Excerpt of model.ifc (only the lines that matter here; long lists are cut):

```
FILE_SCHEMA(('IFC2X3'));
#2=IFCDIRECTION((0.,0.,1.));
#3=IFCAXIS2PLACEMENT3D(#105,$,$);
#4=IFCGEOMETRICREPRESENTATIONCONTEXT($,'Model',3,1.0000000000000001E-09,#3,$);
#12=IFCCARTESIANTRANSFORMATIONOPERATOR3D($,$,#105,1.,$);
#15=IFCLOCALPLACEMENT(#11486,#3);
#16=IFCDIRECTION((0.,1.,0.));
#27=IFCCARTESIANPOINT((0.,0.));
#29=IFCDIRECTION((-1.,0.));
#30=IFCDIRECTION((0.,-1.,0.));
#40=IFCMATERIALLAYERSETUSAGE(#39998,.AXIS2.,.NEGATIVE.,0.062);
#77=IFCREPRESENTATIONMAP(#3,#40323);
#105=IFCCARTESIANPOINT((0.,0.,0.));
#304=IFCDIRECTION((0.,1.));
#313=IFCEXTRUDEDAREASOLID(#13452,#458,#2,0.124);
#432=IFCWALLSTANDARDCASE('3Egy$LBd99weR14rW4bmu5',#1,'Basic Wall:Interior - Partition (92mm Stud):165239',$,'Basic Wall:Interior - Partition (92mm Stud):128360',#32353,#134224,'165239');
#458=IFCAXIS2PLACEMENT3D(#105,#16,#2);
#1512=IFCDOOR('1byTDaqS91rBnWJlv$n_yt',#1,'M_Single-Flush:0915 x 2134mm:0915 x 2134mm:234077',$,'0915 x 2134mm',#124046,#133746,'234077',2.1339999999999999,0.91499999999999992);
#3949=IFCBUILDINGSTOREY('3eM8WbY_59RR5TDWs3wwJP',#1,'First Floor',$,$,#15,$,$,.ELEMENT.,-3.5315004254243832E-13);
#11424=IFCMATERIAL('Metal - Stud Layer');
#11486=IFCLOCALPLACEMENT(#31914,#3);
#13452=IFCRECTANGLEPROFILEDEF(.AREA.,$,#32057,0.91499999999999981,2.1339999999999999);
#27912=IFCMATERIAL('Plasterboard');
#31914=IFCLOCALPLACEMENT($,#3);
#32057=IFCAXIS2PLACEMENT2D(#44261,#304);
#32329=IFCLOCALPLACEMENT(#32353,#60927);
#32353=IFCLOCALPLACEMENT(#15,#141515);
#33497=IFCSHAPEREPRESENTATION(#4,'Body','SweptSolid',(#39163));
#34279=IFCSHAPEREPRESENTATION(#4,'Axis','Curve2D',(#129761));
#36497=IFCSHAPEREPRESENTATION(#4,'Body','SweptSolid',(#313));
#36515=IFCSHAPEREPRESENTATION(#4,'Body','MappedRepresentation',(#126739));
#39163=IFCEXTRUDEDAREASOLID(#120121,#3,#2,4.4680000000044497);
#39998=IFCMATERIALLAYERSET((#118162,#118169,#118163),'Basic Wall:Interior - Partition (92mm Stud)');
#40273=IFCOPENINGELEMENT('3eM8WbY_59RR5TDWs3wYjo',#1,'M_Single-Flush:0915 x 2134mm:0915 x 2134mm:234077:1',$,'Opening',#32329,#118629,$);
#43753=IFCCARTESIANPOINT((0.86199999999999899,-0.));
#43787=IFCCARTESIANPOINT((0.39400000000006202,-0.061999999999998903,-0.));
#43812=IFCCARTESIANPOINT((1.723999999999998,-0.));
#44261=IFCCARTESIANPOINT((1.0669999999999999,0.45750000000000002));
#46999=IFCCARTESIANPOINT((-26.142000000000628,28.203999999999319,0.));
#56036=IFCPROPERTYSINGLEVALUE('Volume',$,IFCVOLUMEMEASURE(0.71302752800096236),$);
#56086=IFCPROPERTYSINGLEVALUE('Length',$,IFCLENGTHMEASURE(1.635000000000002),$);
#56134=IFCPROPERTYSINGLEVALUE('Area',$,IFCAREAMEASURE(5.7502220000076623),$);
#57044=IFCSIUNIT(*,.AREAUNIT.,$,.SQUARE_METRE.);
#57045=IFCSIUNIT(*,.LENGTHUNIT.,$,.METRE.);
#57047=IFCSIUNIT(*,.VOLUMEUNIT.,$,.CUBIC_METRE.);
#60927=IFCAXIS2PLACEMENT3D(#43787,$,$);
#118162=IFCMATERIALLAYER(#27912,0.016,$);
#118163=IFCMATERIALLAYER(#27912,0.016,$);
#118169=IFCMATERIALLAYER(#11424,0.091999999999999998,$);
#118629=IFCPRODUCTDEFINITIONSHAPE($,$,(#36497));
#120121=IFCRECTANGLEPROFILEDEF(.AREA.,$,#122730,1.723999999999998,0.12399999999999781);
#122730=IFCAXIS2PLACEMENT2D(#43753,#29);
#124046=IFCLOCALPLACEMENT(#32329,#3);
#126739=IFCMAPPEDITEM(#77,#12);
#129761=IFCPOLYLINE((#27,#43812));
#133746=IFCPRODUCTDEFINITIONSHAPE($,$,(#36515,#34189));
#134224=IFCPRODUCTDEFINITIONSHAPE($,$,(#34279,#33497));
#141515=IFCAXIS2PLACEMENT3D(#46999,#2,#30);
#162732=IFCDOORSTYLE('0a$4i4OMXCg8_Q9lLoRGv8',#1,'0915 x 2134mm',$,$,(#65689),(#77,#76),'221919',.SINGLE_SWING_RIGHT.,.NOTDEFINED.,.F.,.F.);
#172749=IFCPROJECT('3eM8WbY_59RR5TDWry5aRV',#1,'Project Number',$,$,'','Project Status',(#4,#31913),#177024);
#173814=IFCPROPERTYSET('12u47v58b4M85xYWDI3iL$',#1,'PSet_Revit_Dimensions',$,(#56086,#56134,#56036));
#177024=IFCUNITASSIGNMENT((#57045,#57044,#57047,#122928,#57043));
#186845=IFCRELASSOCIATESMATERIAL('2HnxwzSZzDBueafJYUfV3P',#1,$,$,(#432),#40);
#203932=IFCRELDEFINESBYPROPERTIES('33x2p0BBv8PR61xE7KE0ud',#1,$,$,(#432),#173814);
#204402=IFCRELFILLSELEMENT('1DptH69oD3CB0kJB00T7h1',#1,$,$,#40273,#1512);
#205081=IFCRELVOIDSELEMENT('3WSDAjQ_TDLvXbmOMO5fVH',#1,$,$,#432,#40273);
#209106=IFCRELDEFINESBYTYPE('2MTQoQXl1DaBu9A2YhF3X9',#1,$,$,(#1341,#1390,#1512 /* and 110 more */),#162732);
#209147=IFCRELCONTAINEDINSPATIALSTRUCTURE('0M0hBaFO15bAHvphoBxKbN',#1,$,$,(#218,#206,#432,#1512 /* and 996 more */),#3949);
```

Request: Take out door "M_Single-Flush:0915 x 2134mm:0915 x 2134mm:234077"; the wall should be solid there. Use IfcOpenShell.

```python
import ifcopenshell
import ifcopenshell.api.feature
import ifcopenshell.api.pset
import ifcopenshell.api.root
import ifcopenshell.geom
import ifcopenshell.util.element
import ifcopenshell.util.shape
import ifcopenshell.util.unit

model = ifcopenshell.open("model.ifc")
area_scale = ifcopenshell.util.unit.calculate_unit_scale(model, "AREAUNIT")
volume_scale = ifcopenshell.util.unit.calculate_unit_scale(model, "VOLUMEUNIT")
settings = ifcopenshell.geom.settings()


def volume(element):
    """Net volume in cubic metres, openings subtracted."""
    shape = ifcopenshell.geom.create_shape(settings, element)
    return ifcopenshell.util.shape.get_volume(shape.geometry)


door = model.by_guid("1byTDaqS91rBnWJlv$n_yt")
opening = door.FillsVoids[0].RelatingOpeningElement
wall = opening.VoidsElements[0].RelatingBuildingElement
before = volume(wall)

ifcopenshell.api.root.remove_product(model, product=door)
ifcopenshell.api.feature.remove_feature(model, feature=opening)

after = volume(wall)
thickness = 0.124  # wall thickness in metres

# Update the wall's stored quantities.
pset = model.by_id(ifcopenshell.util.element.get_pset(wall, "PSet_Revit_Dimensions", should_inherit=False)["id"])
ifcopenshell.api.pset.edit_pset(model, pset=pset, properties={
    "Area": model.create_entity("IfcAreaMeasure", after / thickness / area_scale),
    "Volume": model.create_entity("IfcVolumeMeasure", after / volume_scale),
})

print(f"wall volume {before:.3f} -> {after:.3f} m3")

model.write("model-out.ifc")
```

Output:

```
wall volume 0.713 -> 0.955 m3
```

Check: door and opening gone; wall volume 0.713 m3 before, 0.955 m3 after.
